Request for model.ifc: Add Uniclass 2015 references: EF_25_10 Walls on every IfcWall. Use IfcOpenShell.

First a look at what the model holds.

```python
import ifcopenshell

model = ifcopenshell.open("model.ifc")
print(model.schema)
print("classifications:", [c.Name for c in model.by_type("IfcClassification")])
for ifc_class in ("IfcDoor", "IfcRoof", "IfcStair", "IfcWall", "IfcWindow"):
    print(ifc_class, len(model.by_type(ifc_class)))
```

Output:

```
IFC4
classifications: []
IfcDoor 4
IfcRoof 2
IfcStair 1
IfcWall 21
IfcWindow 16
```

```python
import ifcopenshell
import ifcopenshell.api.classification

model = ifcopenshell.open("model.ifc")

system = ifcopenshell.api.classification.add_classification(model, classification="Uniclass 2015")

codes = {
    "IfcWall": ("EF_25_10", "Walls"),
}
for ifc_class, (code, name) in codes.items():
    products = model.by_type(ifc_class)
    ifcopenshell.api.classification.add_reference(
        model, products=products, classification=system, identification=code, name=name
    )
    print(code, len(products))

model.write("model_rev.ifc")
```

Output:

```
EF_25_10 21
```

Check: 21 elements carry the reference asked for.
